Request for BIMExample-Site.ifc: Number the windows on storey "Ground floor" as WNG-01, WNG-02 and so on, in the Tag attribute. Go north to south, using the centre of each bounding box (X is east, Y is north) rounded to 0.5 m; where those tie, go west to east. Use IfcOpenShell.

First a look at what the model holds.

```python
import ifcopenshell
import ifcopenshell.util.element
import ifcopenshell.util.placement

model = ifcopenshell.open("BIMExample-Site.ifc")
print(model.schema)
storey = next(s for s in model.by_type("IfcBuildingStorey") if s.Name == "Ground floor")
windows = [e for e in ifcopenshell.util.element.get_decomposition(storey) if e.is_a("IfcWindow")]
for e in sorted(windows, key=lambda e: e.id()):
    origin = ifcopenshell.util.placement.get_local_placement(e.ObjectPlacement)[:3, 3]
    print(e.id(), e.Tag, e.Name, origin.round(2) + 0.0, sep=" | ")
```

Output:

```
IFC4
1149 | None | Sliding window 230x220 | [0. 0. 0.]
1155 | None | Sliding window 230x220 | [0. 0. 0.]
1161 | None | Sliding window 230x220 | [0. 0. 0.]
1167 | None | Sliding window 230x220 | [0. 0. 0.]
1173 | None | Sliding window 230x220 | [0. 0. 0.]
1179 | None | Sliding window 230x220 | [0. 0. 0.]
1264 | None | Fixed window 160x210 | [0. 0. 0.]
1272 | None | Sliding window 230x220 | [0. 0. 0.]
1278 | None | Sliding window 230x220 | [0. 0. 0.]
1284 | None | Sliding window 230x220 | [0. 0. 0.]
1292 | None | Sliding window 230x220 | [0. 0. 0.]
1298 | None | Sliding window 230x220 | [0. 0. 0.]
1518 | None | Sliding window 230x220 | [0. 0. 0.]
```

```python
import ifcopenshell
import ifcopenshell.geom
import ifcopenshell.util.element
import ifcopenshell.util.shape

model = ifcopenshell.open("BIMExample-Site.ifc")
settings = ifcopenshell.geom.settings()
settings.set("use-world-coords", True)


def centre(element):
    shape = ifcopenshell.geom.create_shape(settings, element)
    return ifcopenshell.util.shape.get_bbox_centroid(shape.geometry)


storey = next(s for s in model.by_type("IfcBuildingStorey") if s.Name == "Ground floor")
windows = [e for e in ifcopenshell.util.element.get_decomposition(storey) if e.is_a("IfcWindow")]

# Insertion points can sit at a corner or the storey origin, so sort by the geometry (in metres).
centres = {e: centre(e) for e in windows}
windows.sort(key=lambda e: (-round(centres[e][1] / 0.5), centres[e][0]))

for i, e in enumerate(windows, start=1):
    number = f"WNG-{i:02d}"
    e.Tag = number
    print(e.id(), number)

model.write("BIMExample-Site-out.ifc")
```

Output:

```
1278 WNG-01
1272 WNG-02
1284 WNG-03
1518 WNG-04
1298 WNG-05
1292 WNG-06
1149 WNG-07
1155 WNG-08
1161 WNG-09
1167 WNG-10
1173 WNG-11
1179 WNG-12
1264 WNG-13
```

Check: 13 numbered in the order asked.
